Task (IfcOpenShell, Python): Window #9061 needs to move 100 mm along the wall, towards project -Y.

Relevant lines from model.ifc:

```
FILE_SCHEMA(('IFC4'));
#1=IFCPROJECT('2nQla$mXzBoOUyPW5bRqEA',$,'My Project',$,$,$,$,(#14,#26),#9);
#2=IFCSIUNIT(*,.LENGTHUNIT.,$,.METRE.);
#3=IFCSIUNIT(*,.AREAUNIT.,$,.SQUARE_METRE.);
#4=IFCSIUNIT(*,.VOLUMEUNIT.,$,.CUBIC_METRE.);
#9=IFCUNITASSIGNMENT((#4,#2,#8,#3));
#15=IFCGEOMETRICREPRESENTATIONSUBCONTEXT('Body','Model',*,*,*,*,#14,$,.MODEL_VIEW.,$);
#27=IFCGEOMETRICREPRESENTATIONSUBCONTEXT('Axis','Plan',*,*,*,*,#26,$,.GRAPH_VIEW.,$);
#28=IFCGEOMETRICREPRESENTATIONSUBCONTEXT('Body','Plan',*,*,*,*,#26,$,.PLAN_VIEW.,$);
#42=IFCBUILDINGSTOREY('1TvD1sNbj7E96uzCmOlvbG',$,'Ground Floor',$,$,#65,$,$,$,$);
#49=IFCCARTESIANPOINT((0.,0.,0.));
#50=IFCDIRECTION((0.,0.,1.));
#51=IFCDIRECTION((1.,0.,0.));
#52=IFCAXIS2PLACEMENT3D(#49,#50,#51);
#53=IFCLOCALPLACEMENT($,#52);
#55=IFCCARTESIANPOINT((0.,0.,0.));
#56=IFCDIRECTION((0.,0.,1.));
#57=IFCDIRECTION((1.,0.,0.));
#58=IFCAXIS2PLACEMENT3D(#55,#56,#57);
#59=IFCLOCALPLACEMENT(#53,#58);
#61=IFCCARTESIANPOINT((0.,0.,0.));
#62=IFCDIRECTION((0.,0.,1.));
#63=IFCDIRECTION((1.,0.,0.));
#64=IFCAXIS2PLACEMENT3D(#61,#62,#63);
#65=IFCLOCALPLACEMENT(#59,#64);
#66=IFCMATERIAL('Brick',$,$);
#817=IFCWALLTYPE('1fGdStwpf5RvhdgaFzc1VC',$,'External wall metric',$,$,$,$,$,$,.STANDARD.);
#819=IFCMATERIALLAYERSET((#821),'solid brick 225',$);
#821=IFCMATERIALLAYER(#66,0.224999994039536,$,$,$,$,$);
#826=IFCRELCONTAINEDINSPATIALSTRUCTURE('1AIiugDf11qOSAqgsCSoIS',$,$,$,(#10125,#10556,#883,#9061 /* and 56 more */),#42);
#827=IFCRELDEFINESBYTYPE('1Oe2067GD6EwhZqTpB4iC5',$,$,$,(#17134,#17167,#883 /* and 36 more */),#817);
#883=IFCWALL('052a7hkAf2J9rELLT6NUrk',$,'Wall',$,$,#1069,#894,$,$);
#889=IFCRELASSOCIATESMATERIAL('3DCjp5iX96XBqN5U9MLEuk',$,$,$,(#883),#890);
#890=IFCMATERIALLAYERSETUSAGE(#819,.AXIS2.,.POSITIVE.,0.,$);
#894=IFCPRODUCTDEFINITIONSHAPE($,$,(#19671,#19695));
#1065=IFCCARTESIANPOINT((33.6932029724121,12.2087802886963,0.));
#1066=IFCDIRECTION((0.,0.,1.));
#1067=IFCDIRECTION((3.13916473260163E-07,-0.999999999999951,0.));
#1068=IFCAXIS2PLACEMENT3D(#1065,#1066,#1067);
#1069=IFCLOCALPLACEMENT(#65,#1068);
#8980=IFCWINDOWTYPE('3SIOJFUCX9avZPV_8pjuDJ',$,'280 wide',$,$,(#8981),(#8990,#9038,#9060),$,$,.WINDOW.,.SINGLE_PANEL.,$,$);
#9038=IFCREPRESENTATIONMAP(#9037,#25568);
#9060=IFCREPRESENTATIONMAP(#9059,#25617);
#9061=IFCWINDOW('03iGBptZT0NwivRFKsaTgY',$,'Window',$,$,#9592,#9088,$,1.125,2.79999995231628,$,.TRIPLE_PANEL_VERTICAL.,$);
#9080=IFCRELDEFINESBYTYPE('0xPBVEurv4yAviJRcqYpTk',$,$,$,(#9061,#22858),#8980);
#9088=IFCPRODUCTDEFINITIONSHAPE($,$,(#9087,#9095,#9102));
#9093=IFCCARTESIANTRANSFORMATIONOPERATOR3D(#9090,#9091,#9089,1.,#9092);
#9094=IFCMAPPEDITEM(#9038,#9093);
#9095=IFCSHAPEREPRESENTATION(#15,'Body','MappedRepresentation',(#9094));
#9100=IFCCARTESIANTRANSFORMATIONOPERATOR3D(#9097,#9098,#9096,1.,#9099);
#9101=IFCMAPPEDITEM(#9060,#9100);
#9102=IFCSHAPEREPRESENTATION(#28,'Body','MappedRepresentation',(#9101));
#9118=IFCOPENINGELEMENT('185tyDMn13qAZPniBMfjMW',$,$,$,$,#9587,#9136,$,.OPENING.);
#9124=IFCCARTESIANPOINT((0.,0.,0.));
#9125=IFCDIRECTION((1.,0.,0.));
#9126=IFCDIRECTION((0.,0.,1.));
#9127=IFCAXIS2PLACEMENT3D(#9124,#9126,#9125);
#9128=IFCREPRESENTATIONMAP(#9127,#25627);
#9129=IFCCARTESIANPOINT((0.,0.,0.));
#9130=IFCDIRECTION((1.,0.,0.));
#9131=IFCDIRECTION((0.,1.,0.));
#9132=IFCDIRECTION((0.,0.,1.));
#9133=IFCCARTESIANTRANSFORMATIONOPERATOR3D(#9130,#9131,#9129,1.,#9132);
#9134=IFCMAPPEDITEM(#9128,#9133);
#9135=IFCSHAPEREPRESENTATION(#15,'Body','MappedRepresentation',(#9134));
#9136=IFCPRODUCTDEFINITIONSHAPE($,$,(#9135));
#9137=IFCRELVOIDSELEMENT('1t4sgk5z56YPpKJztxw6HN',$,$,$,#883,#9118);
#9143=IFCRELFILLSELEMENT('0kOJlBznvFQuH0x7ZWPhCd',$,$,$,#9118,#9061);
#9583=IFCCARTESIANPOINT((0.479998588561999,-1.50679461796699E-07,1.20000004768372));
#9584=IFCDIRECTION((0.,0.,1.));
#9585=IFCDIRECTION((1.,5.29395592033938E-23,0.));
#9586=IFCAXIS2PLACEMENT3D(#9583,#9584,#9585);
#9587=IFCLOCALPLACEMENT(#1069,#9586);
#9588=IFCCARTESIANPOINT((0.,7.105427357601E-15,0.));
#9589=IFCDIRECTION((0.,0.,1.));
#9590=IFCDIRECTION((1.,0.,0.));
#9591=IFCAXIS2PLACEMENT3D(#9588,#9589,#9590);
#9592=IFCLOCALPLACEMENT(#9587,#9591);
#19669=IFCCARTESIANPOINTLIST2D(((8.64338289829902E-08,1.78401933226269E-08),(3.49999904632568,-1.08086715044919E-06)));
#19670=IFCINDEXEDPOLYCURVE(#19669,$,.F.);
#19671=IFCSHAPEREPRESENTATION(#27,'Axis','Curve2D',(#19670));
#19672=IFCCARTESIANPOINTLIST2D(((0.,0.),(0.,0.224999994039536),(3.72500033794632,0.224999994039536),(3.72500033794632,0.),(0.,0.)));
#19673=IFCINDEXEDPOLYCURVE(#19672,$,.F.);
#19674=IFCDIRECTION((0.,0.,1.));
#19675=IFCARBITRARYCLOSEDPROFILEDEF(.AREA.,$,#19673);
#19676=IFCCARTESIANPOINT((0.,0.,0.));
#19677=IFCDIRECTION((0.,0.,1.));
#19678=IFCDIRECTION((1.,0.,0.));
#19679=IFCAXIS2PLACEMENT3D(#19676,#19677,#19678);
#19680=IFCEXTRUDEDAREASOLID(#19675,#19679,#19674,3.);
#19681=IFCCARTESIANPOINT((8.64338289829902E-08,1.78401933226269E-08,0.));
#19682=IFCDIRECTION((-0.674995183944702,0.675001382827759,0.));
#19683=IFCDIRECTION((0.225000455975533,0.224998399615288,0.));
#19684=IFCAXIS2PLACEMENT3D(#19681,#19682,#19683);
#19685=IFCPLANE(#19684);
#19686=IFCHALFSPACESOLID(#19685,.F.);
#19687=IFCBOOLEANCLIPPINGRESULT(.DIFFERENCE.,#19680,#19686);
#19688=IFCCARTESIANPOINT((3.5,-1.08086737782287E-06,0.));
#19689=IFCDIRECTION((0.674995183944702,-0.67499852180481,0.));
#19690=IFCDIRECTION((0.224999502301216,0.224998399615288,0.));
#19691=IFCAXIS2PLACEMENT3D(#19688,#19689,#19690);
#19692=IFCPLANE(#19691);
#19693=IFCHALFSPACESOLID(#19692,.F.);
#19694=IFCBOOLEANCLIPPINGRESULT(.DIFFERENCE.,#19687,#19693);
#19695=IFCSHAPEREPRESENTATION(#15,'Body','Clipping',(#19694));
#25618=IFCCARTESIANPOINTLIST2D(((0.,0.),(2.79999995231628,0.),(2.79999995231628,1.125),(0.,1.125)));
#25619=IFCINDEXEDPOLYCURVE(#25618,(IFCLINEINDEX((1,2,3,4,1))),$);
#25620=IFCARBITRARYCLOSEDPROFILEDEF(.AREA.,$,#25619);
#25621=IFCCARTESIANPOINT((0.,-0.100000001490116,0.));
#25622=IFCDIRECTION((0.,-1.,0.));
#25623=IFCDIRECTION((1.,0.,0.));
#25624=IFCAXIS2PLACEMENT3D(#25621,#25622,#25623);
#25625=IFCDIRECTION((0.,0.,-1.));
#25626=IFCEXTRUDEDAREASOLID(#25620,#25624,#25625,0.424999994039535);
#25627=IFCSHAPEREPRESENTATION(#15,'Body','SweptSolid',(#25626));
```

```python
import ifcopenshell
import ifcopenshell.api.geometry
import ifcopenshell.util.placement
import ifcopenshell.util.unit

model = ifcopenshell.open("model.ifc")
unit_scale = ifcopenshell.util.unit.calculate_unit_scale(model)

window = model.by_guid("03iGBptZT0NwivRFKsaTgY")
opening = window.FillsVoids[0].RelatingOpeningElement
wall = opening.VoidsElements[0].RelatingBuildingElement

wall_matrix = ifcopenshell.util.placement.get_local_placement(wall.ObjectPlacement)
shift = wall_matrix[:3, 0] * 0.1 / unit_scale
before = ifcopenshell.util.placement.get_local_placement(window.ObjectPlacement)[:3, 3].copy()

# The window is placed relative to its opening, so it follows when the opening moves.
matrix = ifcopenshell.util.placement.get_local_placement(opening.ObjectPlacement)
matrix[:3, 3] += shift
ifcopenshell.api.geometry.edit_object_placement(
    model, product=opening, matrix=matrix, is_si=False, should_transform_children=True
)

after = ifcopenshell.util.placement.get_local_placement(window.ObjectPlacement)[:3, 3]
print("window moved by", (after - before).round(3) + 0.0)

model.write("model_v2.ifc")
```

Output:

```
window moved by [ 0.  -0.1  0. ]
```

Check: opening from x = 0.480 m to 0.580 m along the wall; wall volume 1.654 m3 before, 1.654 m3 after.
